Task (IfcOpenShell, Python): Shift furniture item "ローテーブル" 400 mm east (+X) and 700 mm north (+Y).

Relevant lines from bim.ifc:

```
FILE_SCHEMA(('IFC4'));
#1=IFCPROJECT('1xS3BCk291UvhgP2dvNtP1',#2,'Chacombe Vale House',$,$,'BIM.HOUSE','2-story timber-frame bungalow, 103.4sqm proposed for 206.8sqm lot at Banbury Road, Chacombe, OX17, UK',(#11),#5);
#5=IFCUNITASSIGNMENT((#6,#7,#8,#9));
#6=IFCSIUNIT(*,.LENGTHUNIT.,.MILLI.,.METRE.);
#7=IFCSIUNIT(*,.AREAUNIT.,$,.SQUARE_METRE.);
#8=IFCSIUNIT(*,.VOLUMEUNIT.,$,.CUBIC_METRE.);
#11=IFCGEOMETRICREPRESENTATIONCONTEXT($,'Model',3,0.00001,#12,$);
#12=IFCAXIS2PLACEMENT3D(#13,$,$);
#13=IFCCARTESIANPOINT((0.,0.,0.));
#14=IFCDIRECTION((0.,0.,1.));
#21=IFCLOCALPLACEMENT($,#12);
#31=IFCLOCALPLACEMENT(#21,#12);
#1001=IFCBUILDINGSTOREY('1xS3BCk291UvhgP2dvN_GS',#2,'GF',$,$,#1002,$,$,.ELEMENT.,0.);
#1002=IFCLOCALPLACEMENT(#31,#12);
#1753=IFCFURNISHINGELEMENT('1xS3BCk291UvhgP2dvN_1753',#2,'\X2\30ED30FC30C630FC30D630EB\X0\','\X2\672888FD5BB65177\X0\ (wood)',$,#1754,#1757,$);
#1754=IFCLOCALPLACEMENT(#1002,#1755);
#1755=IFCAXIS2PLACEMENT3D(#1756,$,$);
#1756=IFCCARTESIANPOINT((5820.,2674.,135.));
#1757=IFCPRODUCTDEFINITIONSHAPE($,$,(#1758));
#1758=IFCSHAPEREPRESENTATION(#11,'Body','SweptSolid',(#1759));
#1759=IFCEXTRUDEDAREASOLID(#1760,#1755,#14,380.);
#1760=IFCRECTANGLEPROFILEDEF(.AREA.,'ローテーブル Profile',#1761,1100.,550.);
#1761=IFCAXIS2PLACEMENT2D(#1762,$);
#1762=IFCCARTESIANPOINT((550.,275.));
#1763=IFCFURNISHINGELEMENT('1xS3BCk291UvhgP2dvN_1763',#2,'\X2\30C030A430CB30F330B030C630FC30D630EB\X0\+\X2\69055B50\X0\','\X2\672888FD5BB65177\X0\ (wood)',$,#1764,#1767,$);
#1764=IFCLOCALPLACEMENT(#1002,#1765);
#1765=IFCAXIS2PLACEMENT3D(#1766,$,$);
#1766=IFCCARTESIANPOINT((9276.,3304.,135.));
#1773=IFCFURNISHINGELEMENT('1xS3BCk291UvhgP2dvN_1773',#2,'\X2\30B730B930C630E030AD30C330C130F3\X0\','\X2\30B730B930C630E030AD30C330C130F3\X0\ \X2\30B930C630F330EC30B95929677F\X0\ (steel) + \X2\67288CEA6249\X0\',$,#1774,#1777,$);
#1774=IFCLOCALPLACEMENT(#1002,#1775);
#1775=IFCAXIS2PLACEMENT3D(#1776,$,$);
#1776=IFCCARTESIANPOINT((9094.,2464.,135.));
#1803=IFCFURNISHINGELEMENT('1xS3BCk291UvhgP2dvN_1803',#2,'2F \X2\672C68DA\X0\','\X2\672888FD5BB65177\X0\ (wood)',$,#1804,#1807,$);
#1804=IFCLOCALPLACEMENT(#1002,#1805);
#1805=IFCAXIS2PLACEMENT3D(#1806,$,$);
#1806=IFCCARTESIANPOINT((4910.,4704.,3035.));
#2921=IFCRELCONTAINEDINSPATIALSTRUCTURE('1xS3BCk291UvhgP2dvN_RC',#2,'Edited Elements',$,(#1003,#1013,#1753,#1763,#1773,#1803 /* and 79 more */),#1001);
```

```python
import ifcopenshell
import ifcopenshell.api.geometry
import ifcopenshell.util.placement

model = ifcopenshell.open("bim.ifc")

item = model.by_guid("1xS3BCk291UvhgP2dvN_1753")
matrix = ifcopenshell.util.placement.get_local_placement(item.ObjectPlacement)
matrix[0, 3] += 400.0
matrix[1, 3] += 700.0
ifcopenshell.api.geometry.edit_object_placement(model, product=item, matrix=matrix, is_si=False)

print(ifcopenshell.util.placement.get_local_placement(item.ObjectPlacement).round(3) + 0.0)

model.write("bim_v2.ifc")
```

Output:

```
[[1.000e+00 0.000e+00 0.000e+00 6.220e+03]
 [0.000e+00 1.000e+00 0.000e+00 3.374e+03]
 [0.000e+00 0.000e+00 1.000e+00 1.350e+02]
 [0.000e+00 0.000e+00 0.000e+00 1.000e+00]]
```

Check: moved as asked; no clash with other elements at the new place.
